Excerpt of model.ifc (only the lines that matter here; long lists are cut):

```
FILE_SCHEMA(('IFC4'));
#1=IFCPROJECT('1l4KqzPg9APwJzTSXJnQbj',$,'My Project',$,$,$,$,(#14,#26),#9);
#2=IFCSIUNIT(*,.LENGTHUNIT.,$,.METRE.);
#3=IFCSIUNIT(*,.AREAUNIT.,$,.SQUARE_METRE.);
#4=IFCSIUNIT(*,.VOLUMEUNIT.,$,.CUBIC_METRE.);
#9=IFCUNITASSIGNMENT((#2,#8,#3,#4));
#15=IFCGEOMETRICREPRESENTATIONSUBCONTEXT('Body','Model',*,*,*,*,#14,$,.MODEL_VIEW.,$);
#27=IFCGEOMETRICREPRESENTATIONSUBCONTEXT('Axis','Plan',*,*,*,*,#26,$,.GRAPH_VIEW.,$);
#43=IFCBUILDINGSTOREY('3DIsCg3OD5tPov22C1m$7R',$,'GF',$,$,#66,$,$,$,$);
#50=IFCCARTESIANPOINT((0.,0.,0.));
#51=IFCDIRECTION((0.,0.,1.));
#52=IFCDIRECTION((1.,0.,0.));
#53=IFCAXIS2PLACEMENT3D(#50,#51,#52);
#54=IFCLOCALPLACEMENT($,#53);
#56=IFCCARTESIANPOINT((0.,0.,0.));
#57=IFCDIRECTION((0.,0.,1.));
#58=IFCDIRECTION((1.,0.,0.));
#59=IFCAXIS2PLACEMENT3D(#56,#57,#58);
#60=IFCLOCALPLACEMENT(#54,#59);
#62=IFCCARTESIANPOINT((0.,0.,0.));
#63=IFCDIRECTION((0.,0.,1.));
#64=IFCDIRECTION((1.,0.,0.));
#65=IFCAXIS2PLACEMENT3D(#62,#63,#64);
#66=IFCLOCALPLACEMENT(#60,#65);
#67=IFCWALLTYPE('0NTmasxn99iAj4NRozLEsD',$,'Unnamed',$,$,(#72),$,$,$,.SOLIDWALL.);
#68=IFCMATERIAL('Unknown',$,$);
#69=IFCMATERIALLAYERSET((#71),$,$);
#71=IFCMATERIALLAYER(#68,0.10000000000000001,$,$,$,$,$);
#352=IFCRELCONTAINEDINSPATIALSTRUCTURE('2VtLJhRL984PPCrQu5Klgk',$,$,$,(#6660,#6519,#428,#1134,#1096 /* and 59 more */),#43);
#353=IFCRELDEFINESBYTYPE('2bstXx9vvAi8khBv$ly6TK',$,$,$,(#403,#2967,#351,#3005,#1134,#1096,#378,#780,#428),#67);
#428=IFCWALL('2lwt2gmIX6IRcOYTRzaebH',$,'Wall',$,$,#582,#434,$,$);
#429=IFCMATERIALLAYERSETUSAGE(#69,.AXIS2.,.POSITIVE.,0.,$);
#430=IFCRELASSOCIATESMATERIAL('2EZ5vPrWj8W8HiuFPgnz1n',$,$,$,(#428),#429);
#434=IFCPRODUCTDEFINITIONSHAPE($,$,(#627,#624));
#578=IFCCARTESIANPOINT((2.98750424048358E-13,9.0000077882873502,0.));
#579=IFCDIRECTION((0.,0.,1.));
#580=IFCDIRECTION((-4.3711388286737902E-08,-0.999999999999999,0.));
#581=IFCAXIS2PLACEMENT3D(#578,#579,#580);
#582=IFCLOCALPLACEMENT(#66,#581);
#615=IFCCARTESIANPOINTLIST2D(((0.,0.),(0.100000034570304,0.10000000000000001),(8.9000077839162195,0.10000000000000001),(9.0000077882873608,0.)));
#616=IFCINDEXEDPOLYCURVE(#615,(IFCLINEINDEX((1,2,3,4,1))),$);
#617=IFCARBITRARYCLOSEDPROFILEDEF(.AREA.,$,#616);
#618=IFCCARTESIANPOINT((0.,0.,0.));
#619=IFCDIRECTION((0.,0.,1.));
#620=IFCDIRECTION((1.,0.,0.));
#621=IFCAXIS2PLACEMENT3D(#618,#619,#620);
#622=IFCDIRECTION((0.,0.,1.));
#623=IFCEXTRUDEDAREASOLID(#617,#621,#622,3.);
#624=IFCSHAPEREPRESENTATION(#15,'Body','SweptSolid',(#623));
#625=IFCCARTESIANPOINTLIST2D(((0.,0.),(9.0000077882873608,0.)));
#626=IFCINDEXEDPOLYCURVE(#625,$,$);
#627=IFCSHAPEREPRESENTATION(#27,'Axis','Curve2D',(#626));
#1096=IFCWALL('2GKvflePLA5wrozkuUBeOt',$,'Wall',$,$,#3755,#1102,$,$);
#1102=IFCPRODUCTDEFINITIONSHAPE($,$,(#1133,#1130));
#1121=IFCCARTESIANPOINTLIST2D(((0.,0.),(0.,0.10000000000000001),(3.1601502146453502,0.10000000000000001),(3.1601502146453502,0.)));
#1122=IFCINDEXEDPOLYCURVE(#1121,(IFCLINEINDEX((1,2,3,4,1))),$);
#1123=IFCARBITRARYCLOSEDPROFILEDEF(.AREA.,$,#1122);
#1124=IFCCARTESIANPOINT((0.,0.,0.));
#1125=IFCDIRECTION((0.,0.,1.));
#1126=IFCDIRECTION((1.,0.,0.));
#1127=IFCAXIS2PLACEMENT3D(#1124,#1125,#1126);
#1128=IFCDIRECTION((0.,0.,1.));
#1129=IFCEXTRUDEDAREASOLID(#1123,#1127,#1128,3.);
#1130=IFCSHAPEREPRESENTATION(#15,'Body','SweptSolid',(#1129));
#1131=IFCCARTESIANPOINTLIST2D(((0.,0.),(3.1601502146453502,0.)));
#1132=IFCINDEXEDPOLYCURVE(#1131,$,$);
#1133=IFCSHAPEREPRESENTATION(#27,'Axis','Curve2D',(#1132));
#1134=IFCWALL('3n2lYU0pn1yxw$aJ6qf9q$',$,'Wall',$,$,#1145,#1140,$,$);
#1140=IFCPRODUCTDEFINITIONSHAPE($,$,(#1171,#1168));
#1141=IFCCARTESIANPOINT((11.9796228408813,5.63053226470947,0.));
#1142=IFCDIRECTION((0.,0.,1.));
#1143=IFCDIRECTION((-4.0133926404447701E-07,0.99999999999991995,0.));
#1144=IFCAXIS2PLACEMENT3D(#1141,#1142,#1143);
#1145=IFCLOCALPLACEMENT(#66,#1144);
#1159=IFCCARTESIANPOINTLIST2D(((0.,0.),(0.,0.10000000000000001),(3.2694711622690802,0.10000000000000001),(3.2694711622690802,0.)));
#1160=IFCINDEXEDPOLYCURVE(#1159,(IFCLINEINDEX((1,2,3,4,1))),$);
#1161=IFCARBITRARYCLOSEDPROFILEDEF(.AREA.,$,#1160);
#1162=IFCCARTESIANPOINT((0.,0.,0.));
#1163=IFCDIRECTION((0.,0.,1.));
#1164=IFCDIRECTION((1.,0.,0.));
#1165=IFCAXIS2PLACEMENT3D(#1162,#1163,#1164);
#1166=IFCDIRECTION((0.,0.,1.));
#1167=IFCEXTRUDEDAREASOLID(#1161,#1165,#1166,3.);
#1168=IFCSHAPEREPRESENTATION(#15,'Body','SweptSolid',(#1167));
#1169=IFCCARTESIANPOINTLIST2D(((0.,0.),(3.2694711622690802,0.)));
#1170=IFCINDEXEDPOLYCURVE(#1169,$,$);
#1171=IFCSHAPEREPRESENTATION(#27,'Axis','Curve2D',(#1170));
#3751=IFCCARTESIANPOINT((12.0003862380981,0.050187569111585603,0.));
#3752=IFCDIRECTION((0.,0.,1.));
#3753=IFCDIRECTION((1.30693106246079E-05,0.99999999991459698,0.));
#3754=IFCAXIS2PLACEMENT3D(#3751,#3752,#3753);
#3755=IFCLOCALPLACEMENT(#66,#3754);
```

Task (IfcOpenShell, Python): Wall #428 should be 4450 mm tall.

```python
import ifcopenshell
import ifcopenshell.geom
import ifcopenshell.util.representation
import ifcopenshell.util.shape
import ifcopenshell.util.unit

model = ifcopenshell.open("model.ifc")
unit_scale = ifcopenshell.util.unit.calculate_unit_scale(model)
settings = ifcopenshell.geom.settings()


def volume(element):
    """Net volume in cubic metres, openings subtracted."""
    shape = ifcopenshell.geom.create_shape(settings, element)
    return ifcopenshell.util.shape.get_volume(shape.geometry)


wall = model.by_id(428)
before = volume(wall)

body = ifcopenshell.util.representation.get_representation(wall, "Model", "Body")
solid = body.Items[0]
old_height = solid.Depth
solid.Depth = 4.45 / unit_scale
after = volume(wall)

print(f"height {old_height:g} -> {solid.Depth:g}, volume {before:.3f} -> {after:.3f} m3")

model.write("model_edited.ifc")
```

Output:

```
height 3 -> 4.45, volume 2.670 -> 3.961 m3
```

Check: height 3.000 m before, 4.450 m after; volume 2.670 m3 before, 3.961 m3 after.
